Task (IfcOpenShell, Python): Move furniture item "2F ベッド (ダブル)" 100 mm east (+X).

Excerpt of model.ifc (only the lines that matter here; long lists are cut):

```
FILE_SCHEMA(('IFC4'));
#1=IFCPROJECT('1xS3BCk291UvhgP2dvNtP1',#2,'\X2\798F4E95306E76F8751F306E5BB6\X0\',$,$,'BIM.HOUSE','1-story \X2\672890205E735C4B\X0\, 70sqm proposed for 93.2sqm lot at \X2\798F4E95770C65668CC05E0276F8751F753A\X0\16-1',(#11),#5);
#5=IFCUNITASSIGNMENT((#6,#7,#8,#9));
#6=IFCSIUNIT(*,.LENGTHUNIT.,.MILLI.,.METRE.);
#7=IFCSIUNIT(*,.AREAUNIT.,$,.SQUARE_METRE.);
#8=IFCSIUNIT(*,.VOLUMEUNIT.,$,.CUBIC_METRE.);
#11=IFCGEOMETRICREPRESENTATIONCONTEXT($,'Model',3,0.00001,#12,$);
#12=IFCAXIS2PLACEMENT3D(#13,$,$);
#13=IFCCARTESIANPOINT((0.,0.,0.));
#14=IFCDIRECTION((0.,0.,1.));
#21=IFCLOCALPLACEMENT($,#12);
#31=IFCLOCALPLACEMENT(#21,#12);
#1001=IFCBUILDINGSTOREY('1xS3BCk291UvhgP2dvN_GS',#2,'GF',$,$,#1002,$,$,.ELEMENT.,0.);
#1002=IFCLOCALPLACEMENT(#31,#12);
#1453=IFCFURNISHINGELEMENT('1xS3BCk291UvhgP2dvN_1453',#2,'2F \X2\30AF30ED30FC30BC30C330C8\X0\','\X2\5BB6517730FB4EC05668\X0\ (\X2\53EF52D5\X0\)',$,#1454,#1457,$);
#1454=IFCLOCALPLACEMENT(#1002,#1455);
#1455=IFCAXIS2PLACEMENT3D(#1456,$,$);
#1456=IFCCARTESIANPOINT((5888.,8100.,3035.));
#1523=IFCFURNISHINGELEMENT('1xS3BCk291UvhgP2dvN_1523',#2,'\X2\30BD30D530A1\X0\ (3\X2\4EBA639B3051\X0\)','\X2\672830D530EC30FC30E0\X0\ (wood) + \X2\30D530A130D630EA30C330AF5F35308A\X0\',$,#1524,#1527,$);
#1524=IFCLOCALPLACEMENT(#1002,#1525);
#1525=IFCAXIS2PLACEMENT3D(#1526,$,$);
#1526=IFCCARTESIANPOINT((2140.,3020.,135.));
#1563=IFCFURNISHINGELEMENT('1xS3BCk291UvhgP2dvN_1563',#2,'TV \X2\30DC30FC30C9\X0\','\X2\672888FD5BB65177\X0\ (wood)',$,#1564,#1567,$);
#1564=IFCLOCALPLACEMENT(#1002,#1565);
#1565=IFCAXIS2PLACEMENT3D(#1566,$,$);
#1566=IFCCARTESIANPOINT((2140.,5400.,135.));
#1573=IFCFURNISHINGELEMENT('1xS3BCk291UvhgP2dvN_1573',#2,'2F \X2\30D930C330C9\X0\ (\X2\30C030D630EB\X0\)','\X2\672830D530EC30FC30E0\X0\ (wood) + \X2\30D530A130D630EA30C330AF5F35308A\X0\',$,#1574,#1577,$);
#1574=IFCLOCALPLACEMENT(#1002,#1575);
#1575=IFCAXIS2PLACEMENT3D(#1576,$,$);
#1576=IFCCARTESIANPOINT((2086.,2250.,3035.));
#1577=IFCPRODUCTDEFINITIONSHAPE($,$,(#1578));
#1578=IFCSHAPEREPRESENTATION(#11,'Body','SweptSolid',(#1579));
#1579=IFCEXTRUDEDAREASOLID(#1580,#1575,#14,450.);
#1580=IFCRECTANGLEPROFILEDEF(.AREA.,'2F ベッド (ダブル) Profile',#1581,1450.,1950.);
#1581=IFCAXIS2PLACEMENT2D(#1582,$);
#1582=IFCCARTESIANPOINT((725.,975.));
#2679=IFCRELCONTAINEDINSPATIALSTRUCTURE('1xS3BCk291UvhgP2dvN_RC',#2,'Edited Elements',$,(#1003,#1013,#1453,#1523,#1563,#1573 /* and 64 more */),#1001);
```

```python
import ifcopenshell
import ifcopenshell.api.geometry
import ifcopenshell.util.placement
import ifcopenshell.util.unit

model = ifcopenshell.open("model.ifc")
unit_scale = ifcopenshell.util.unit.calculate_unit_scale(model)

item = model.by_id(1573)
matrix = ifcopenshell.util.placement.get_local_placement(item.ObjectPlacement)
matrix[0, 3] += 0.1 / unit_scale
ifcopenshell.api.geometry.edit_object_placement(model, product=item, matrix=matrix, is_si=False)

print(ifcopenshell.util.placement.get_local_placement(item.ObjectPlacement).round(3) + 0.0)

model.write("model-out.ifc")
```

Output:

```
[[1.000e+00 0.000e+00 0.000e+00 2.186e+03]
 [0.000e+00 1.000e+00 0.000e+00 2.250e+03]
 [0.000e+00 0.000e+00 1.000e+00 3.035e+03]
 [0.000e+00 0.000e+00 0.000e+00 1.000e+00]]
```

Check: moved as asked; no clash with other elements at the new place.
